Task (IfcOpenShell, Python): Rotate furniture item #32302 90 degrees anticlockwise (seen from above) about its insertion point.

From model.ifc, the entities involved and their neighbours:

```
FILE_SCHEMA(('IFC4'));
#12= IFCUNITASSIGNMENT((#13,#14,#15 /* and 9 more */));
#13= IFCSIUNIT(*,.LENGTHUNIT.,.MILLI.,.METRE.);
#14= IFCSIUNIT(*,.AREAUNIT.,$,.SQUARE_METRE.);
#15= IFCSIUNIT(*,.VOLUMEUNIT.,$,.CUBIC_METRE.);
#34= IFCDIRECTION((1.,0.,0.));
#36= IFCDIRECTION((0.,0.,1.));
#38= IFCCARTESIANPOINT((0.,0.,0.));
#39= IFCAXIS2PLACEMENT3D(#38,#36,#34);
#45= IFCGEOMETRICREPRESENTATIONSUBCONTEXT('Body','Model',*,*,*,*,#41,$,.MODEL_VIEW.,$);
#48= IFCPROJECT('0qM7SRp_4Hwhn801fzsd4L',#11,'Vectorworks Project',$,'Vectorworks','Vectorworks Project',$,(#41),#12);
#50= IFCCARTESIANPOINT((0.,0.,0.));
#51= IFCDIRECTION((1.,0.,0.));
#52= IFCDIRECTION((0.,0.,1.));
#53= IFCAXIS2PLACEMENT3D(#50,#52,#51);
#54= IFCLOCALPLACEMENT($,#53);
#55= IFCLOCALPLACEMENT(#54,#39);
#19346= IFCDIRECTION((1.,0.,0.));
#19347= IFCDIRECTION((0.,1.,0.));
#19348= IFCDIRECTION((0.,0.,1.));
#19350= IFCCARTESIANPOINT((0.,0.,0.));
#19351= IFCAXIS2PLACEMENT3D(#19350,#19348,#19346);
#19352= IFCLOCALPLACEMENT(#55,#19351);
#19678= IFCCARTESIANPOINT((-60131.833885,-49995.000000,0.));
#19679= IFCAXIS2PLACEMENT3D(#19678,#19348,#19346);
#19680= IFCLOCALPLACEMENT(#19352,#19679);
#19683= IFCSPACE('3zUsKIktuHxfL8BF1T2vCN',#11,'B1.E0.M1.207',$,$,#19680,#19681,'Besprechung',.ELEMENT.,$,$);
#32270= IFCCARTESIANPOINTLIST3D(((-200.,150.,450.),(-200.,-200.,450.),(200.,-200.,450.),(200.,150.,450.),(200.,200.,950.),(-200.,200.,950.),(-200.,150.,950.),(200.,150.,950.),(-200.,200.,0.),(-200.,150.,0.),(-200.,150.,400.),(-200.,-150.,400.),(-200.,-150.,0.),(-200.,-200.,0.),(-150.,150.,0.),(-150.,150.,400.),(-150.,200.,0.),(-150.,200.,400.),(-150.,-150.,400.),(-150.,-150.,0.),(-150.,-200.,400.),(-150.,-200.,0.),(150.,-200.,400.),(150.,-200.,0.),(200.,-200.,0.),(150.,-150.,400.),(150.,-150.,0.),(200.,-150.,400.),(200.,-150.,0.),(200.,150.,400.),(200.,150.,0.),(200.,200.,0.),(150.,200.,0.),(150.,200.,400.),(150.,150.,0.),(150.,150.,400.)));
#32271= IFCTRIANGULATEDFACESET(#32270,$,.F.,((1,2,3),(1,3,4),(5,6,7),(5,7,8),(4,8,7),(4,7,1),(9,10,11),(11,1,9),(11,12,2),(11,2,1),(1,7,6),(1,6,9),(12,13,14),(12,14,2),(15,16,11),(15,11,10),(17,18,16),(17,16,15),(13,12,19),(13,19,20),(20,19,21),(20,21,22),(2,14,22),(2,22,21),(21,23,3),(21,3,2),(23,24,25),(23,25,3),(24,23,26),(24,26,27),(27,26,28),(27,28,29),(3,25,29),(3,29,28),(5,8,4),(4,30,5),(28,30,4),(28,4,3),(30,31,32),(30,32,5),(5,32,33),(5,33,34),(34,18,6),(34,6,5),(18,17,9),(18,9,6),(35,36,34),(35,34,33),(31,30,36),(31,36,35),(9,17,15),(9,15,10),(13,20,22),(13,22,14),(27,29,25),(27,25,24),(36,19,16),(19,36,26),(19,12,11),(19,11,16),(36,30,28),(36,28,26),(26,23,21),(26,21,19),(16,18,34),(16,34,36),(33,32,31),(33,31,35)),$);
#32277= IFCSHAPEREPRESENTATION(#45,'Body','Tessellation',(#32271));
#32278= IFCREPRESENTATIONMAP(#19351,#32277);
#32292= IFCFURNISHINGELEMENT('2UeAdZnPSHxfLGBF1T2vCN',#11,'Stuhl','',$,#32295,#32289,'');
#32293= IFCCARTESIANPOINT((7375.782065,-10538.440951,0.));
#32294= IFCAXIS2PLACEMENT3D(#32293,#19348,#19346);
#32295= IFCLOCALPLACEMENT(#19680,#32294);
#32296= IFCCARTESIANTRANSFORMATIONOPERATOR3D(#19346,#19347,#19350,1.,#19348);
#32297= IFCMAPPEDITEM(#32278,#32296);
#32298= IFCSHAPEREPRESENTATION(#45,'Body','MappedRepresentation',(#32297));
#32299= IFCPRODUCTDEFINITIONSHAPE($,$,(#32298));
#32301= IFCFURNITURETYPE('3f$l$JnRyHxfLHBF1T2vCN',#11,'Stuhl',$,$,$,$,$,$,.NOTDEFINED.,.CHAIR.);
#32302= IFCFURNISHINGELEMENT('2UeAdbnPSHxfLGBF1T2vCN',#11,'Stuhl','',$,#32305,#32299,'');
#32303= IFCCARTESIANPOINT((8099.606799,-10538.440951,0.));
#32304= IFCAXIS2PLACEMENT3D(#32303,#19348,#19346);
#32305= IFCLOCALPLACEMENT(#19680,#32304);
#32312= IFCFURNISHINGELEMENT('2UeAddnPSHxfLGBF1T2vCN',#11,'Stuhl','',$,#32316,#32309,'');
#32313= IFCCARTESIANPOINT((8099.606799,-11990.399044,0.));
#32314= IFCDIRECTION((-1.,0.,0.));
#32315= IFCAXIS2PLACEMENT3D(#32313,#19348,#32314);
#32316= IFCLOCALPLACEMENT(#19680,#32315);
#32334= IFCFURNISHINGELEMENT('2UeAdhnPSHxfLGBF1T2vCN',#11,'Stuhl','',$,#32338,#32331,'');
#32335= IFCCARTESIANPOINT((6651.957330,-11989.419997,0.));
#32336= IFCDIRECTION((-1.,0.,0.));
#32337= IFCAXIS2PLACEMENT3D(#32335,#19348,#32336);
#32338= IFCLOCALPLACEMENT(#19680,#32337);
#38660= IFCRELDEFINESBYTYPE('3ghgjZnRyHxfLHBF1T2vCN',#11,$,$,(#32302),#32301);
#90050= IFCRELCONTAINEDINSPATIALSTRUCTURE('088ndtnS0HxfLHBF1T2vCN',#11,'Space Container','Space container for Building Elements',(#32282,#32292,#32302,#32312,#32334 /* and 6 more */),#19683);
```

```python
import ifcopenshell
import ifcopenshell.api.geometry
import ifcopenshell.util.placement

model = ifcopenshell.open("model.ifc")

item = model.by_guid("2UeAdbnPSHxfLGBF1T2vCN")
matrix = ifcopenshell.util.placement.get_local_placement(item.ObjectPlacement)
matrix = matrix @ ifcopenshell.util.placement.rotation(90, "Z")
ifcopenshell.api.geometry.edit_object_placement(model, product=item, matrix=matrix, is_si=False)

print(ifcopenshell.util.placement.get_local_placement(item.ObjectPlacement).round(3) + 0.0)

model.write("model-out.ifc")
```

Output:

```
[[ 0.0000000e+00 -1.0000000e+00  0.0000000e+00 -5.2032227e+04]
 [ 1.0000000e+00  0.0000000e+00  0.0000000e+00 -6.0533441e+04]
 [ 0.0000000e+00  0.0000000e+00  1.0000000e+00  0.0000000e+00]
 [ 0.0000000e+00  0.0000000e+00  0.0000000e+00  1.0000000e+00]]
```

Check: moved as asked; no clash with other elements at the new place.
